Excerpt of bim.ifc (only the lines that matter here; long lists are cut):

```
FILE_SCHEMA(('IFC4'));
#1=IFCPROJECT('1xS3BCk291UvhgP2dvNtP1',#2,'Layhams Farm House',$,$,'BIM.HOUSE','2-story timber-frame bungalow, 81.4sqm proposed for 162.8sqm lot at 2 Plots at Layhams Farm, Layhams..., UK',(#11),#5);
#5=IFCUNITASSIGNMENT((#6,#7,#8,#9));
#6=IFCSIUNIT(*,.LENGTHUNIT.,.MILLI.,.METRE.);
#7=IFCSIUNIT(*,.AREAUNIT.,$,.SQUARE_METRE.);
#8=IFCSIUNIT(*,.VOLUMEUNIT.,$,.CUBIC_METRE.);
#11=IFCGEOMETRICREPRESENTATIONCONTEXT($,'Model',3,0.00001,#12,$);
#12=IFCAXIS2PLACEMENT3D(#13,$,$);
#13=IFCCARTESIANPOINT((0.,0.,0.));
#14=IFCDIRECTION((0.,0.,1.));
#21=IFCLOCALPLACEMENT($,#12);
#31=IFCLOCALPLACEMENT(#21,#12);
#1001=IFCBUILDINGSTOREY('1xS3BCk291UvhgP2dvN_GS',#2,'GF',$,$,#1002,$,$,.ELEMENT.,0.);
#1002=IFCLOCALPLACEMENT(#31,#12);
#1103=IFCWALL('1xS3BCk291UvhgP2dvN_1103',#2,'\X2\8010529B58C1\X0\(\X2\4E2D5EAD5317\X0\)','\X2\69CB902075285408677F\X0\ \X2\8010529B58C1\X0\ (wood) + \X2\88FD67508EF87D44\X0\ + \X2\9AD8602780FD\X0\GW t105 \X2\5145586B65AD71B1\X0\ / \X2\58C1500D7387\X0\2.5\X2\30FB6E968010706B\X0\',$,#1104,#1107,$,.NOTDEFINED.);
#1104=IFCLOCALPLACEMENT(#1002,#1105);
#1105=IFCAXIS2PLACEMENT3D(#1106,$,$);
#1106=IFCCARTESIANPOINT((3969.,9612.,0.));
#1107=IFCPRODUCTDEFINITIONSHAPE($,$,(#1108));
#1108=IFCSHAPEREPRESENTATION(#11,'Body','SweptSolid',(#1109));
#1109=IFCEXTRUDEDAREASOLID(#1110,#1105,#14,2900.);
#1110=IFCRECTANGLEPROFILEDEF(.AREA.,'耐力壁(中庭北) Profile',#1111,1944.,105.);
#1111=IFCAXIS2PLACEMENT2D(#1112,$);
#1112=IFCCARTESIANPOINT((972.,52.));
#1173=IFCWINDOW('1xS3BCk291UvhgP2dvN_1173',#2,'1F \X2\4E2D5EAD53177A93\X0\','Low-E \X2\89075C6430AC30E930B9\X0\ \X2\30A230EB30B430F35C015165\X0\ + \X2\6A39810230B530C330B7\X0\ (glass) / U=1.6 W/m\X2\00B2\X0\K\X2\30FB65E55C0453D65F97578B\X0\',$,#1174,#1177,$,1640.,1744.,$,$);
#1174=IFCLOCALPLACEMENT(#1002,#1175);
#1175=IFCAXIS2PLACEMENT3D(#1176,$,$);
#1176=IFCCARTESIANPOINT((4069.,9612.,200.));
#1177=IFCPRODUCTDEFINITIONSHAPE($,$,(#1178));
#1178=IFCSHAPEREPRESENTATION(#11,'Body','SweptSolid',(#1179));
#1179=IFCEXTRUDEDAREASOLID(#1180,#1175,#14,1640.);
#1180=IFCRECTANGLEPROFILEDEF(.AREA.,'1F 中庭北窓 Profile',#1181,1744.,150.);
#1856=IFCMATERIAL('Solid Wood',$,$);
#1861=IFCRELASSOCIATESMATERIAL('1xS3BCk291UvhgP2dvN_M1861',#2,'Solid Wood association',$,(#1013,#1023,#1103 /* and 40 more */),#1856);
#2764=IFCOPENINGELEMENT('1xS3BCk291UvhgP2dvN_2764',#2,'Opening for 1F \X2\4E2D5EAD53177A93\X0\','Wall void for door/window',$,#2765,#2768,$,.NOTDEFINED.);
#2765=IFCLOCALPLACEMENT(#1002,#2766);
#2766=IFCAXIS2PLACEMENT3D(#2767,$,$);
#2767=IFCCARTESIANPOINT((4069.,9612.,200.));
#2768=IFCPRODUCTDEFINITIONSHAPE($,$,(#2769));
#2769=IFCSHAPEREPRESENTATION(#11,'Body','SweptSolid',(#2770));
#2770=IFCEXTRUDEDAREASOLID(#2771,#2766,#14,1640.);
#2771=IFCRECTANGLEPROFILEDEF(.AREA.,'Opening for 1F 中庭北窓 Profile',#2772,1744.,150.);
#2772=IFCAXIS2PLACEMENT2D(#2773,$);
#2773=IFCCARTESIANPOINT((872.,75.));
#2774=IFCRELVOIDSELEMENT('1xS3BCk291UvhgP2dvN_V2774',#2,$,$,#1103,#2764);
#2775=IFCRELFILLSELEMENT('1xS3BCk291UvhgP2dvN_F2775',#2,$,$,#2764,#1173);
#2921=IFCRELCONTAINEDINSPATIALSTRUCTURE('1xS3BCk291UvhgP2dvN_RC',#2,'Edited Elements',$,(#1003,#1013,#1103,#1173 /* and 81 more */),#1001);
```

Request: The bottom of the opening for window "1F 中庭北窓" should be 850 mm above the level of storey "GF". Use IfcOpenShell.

```python
import numpy as np
import ifcopenshell
import ifcopenshell.api.geometry
import ifcopenshell.geom
import ifcopenshell.util.element
import ifcopenshell.util.placement
import ifcopenshell.util.shape
import ifcopenshell.util.unit

model = ifcopenshell.open("bim.ifc")
unit_scale = ifcopenshell.util.unit.calculate_unit_scale(model)

window = model.by_guid("1xS3BCk291UvhgP2dvN_1173")
opening = window.FillsVoids[0].RelatingOpeningElement
storey = ifcopenshell.util.element.get_container(window, ifc_class="IfcBuildingStorey")
level = ifcopenshell.util.placement.get_local_placement(storey.ObjectPlacement)[2, 3]

# The opening's origin need not be at the sill, so measure its lowest point.
shape = ifcopenshell.geom.create_shape(ifcopenshell.geom.settings(), opening)
bottom = ifcopenshell.util.shape.get_shape_bottom_elevation(shape, shape.geometry) / unit_scale
dz = level + 0.85 / unit_scale - bottom

shift = np.array([0.0, 0.0, dz])
# The window is not placed relative to its opening, so move both.
for product in (opening, window):
    matrix = ifcopenshell.util.placement.get_local_placement(product.ObjectPlacement)
    matrix[:3, 3] += shift
    ifcopenshell.api.geometry.edit_object_placement(model, product=product, matrix=matrix, is_si=False)

print(f"moved by {dz * unit_scale:+.3f} m")

model.write("bim_updated.ifc")
```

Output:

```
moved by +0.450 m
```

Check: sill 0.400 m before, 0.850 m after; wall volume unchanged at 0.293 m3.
